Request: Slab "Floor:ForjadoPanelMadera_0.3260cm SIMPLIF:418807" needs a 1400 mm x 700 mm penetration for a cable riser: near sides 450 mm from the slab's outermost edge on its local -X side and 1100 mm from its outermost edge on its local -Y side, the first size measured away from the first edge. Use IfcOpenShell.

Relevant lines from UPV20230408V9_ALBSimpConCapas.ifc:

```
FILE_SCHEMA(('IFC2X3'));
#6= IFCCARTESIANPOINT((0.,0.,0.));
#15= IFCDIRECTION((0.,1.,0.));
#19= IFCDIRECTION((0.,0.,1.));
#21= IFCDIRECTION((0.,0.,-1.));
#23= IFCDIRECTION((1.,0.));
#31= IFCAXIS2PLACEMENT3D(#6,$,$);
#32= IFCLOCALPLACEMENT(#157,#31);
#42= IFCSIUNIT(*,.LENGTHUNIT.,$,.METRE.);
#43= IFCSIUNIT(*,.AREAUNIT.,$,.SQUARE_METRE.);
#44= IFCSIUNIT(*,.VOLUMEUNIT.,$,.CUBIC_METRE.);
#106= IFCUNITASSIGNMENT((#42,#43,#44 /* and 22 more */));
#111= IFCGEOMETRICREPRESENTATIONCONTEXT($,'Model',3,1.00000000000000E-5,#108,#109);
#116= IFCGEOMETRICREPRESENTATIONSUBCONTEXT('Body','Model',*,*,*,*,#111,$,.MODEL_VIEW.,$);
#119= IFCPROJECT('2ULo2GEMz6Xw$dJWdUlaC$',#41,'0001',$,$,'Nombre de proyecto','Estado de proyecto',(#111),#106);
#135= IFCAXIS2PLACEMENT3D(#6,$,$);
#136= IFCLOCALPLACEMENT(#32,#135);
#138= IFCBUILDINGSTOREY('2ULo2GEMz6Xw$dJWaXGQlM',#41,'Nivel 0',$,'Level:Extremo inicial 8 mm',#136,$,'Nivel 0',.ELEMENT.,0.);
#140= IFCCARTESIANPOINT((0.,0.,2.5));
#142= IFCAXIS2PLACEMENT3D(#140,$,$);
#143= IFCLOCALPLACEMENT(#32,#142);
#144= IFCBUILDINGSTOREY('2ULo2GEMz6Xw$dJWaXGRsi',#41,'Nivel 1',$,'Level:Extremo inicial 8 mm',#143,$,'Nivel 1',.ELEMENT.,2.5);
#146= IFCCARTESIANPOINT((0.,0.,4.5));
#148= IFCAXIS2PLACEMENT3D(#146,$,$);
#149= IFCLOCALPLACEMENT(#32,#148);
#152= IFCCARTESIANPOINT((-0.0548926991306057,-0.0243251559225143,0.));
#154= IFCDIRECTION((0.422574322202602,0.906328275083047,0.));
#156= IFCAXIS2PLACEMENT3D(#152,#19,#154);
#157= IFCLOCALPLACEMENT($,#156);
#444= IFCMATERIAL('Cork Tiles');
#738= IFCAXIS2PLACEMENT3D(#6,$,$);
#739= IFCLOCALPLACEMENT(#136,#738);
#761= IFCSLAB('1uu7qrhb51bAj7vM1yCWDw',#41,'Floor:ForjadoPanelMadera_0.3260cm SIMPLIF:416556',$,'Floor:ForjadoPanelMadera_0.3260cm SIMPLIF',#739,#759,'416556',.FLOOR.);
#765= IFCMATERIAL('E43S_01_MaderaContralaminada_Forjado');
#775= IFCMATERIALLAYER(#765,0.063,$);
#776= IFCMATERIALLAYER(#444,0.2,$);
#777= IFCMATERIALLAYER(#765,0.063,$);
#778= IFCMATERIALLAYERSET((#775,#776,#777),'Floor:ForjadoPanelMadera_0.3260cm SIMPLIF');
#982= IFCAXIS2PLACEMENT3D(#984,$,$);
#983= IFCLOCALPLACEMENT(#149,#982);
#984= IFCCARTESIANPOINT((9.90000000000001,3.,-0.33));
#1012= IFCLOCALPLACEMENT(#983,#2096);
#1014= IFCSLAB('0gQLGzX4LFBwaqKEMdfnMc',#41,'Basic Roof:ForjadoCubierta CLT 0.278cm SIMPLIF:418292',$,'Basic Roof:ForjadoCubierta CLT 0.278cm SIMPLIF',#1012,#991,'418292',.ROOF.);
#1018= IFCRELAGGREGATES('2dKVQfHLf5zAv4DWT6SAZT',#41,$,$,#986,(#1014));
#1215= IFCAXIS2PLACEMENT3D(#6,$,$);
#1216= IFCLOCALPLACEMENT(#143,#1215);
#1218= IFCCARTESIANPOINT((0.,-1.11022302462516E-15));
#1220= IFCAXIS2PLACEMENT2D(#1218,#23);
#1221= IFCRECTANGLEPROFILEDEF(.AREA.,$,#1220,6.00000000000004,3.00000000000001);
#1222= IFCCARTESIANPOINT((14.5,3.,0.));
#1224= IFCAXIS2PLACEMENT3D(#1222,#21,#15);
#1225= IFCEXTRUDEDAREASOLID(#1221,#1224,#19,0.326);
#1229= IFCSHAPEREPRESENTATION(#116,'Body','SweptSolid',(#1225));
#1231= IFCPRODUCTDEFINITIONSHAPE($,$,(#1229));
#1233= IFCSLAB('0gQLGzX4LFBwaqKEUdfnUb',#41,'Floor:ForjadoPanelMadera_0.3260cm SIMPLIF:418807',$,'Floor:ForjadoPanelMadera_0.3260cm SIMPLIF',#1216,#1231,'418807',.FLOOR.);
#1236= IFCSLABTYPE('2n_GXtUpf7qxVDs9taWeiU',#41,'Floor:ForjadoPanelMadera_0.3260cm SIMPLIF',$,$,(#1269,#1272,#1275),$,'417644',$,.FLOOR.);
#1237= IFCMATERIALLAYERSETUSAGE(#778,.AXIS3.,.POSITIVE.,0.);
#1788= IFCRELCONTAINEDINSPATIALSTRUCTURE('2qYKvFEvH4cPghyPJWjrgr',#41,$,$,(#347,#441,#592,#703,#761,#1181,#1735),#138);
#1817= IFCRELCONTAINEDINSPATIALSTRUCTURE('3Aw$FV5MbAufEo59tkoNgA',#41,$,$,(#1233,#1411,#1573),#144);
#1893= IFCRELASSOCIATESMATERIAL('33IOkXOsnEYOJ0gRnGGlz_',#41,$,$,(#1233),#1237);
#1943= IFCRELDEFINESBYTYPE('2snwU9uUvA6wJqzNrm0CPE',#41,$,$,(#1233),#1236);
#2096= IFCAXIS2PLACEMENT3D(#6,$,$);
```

```python
import numpy as np
import ifcopenshell
import ifcopenshell.api.feature
import ifcopenshell.api.geometry
import ifcopenshell.api.root
import ifcopenshell.geom
import ifcopenshell.util.placement
import ifcopenshell.util.representation
import ifcopenshell.util.shape
import ifcopenshell.util.unit

model = ifcopenshell.open("UPV20230408V9_ALBSimpConCapas.ifc")
unit_scale = ifcopenshell.util.unit.calculate_unit_scale(model)
settings = ifcopenshell.geom.settings()


def volume(element):
    """Net volume in cubic metres, openings subtracted."""
    shape = ifcopenshell.geom.create_shape(settings, element)
    return ifcopenshell.util.shape.get_volume(shape.geometry)


slab = model.by_id(1233)
before = volume(slab)

# Extent in the slab's own axes, in metres. The edges named are its -X and -Y sides.
slab_shape = ifcopenshell.geom.create_shape(settings, slab)
vertices = ifcopenshell.util.shape.get_vertices(slab_shape.geometry)
x_min, y_min, bottom = vertices.min(axis=0)
top = vertices[:, 2].max()

opening = ifcopenshell.api.root.create_entity(model, ifc_class="IfcOpeningElement", name="Cable riser opening")
context = ifcopenshell.util.representation.get_context(model, "Model", "Body", "MODEL_VIEW")
width, depth = 1.4, 0.7
outline = [(0.0, 0.0), (width, 0.0), (width, depth), (0.0, depth), (0.0, 0.0)]
# Overshoot both faces by 50 mm so the cut is clean.
shape = ifcopenshell.api.geometry.add_slab_representation(
    model, context=context, depth=top - bottom + 0.1, polyline=outline
)
ifcopenshell.api.geometry.assign_representation(model, product=opening, representation=shape)

matrix = ifcopenshell.util.placement.get_local_placement(slab.ObjectPlacement)
matrix[:, 3] = matrix @ np.append(np.array([x_min + 0.45, y_min + 1.1, bottom - 0.05]) / unit_scale, 1.0)
ifcopenshell.api.geometry.edit_object_placement(model, product=opening, matrix=matrix, is_si=False)
ifcopenshell.api.feature.add_feature(model, feature=opening, element=slab)

after = volume(slab)

print(f"slab volume {before:.3f} -> {after:.3f} m3")

model.write("UPV20230408V9_ALBSimpConCapas_edited.ifc")
```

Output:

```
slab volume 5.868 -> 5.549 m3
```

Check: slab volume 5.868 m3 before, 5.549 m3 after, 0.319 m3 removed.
